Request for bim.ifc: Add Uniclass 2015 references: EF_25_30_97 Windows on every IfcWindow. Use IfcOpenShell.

First a look at what the model holds.

```python
import ifcopenshell

model = ifcopenshell.open("bim.ifc")
print(model.schema)
print("classifications:", [c.Name for c in model.by_type("IfcClassification")])
for ifc_class in ("IfcDoor", "IfcRoof", "IfcStair", "IfcWall", "IfcWindow"):
    print(ifc_class, len(model.by_type(ifc_class)))
```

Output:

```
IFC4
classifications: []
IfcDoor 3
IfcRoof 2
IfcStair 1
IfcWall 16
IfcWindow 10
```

```python
import ifcopenshell
import ifcopenshell.api.classification

model = ifcopenshell.open("bim.ifc")

system = ifcopenshell.api.classification.add_classification(model, classification="Uniclass 2015")

codes = {
    "IfcWindow": ("EF_25_30_97", "Windows"),
}
for ifc_class, (code, name) in codes.items():
    products = model.by_type(ifc_class)
    ifcopenshell.api.classification.add_reference(
        model, products=products, classification=system, identification=code, name=name
    )
    print(code, len(products))

model.write("bim_edited.ifc")
```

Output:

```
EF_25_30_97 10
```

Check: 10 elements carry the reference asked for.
